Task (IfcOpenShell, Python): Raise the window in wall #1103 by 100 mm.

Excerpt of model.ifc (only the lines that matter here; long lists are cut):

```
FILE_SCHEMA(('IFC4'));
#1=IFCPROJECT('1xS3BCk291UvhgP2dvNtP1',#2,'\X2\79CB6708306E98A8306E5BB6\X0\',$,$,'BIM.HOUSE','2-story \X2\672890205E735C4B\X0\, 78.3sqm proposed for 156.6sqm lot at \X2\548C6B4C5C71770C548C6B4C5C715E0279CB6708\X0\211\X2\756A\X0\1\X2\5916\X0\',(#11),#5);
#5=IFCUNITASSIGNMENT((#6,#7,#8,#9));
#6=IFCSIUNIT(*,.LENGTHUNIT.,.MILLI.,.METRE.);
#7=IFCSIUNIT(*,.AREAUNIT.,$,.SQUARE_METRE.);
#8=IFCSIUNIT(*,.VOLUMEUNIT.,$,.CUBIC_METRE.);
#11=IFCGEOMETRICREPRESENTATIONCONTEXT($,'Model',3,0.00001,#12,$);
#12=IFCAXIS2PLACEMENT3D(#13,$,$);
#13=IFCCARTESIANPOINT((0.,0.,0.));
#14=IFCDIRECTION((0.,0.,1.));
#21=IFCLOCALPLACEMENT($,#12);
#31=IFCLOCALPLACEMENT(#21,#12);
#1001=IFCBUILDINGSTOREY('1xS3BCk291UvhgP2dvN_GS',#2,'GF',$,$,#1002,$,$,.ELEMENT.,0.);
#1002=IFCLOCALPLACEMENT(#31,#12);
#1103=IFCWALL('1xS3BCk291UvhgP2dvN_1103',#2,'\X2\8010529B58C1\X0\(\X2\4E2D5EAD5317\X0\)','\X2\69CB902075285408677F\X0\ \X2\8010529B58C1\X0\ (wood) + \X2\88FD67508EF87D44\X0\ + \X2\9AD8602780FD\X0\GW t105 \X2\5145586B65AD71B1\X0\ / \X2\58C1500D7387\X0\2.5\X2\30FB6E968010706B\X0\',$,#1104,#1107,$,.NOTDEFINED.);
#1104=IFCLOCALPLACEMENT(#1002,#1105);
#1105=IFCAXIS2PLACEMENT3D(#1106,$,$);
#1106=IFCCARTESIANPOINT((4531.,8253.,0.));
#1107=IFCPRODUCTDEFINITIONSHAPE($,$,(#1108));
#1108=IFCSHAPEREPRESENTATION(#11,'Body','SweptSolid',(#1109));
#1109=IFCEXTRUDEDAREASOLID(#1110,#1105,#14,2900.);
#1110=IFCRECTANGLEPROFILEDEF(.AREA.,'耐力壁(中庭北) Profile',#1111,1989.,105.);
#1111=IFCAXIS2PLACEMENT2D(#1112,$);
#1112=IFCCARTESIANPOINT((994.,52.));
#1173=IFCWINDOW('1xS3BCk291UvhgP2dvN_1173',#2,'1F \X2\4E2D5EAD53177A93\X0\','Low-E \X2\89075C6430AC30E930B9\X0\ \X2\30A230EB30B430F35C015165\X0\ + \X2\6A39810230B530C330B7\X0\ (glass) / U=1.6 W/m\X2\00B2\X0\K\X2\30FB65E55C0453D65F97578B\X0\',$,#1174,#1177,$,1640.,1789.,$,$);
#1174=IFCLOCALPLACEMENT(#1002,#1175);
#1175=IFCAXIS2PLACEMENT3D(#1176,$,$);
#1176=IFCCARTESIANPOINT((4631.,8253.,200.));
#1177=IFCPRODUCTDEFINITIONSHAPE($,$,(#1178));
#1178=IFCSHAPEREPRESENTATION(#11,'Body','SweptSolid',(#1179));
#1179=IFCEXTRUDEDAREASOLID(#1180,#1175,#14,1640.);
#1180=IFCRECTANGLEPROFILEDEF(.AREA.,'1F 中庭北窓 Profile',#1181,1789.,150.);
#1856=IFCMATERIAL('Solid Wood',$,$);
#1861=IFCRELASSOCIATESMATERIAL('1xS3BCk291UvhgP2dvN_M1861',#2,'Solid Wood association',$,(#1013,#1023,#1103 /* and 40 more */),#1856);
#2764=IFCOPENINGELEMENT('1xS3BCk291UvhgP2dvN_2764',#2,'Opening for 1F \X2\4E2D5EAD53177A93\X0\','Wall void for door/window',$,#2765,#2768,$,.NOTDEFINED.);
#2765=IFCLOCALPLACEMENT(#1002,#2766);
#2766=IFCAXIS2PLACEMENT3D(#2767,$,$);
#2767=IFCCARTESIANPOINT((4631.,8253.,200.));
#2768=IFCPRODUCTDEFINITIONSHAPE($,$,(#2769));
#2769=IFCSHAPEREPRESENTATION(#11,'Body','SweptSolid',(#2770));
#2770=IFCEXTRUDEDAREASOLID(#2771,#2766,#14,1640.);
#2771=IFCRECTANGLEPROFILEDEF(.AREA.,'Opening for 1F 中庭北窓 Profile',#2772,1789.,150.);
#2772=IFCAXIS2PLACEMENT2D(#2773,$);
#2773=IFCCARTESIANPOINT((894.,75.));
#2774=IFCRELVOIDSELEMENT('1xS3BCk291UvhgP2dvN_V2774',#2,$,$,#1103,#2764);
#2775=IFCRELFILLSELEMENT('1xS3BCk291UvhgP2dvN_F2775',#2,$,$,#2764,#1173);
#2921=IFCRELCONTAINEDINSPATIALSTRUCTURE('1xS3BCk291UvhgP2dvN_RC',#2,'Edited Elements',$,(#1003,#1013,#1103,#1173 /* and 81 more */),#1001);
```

```python
import numpy as np
import ifcopenshell
import ifcopenshell.api.geometry
import ifcopenshell.util.placement
import ifcopenshell.util.unit

model = ifcopenshell.open("model.ifc")
unit_scale = ifcopenshell.util.unit.calculate_unit_scale(model)

window = model.by_id(1173)
opening = window.FillsVoids[0].RelatingOpeningElement
dz = 0.1 / unit_scale

shift = np.array([0.0, 0.0, dz])
# The window is not placed relative to its opening, so move both.
for product in (opening, window):
    matrix = ifcopenshell.util.placement.get_local_placement(product.ObjectPlacement)
    matrix[:3, 3] += shift
    ifcopenshell.api.geometry.edit_object_placement(model, product=product, matrix=matrix, is_si=False)

print(f"moved by {dz * unit_scale:+.3f} m")

model.write("model-out.ifc")
```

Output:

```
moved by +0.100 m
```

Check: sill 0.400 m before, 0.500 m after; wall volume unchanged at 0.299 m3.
